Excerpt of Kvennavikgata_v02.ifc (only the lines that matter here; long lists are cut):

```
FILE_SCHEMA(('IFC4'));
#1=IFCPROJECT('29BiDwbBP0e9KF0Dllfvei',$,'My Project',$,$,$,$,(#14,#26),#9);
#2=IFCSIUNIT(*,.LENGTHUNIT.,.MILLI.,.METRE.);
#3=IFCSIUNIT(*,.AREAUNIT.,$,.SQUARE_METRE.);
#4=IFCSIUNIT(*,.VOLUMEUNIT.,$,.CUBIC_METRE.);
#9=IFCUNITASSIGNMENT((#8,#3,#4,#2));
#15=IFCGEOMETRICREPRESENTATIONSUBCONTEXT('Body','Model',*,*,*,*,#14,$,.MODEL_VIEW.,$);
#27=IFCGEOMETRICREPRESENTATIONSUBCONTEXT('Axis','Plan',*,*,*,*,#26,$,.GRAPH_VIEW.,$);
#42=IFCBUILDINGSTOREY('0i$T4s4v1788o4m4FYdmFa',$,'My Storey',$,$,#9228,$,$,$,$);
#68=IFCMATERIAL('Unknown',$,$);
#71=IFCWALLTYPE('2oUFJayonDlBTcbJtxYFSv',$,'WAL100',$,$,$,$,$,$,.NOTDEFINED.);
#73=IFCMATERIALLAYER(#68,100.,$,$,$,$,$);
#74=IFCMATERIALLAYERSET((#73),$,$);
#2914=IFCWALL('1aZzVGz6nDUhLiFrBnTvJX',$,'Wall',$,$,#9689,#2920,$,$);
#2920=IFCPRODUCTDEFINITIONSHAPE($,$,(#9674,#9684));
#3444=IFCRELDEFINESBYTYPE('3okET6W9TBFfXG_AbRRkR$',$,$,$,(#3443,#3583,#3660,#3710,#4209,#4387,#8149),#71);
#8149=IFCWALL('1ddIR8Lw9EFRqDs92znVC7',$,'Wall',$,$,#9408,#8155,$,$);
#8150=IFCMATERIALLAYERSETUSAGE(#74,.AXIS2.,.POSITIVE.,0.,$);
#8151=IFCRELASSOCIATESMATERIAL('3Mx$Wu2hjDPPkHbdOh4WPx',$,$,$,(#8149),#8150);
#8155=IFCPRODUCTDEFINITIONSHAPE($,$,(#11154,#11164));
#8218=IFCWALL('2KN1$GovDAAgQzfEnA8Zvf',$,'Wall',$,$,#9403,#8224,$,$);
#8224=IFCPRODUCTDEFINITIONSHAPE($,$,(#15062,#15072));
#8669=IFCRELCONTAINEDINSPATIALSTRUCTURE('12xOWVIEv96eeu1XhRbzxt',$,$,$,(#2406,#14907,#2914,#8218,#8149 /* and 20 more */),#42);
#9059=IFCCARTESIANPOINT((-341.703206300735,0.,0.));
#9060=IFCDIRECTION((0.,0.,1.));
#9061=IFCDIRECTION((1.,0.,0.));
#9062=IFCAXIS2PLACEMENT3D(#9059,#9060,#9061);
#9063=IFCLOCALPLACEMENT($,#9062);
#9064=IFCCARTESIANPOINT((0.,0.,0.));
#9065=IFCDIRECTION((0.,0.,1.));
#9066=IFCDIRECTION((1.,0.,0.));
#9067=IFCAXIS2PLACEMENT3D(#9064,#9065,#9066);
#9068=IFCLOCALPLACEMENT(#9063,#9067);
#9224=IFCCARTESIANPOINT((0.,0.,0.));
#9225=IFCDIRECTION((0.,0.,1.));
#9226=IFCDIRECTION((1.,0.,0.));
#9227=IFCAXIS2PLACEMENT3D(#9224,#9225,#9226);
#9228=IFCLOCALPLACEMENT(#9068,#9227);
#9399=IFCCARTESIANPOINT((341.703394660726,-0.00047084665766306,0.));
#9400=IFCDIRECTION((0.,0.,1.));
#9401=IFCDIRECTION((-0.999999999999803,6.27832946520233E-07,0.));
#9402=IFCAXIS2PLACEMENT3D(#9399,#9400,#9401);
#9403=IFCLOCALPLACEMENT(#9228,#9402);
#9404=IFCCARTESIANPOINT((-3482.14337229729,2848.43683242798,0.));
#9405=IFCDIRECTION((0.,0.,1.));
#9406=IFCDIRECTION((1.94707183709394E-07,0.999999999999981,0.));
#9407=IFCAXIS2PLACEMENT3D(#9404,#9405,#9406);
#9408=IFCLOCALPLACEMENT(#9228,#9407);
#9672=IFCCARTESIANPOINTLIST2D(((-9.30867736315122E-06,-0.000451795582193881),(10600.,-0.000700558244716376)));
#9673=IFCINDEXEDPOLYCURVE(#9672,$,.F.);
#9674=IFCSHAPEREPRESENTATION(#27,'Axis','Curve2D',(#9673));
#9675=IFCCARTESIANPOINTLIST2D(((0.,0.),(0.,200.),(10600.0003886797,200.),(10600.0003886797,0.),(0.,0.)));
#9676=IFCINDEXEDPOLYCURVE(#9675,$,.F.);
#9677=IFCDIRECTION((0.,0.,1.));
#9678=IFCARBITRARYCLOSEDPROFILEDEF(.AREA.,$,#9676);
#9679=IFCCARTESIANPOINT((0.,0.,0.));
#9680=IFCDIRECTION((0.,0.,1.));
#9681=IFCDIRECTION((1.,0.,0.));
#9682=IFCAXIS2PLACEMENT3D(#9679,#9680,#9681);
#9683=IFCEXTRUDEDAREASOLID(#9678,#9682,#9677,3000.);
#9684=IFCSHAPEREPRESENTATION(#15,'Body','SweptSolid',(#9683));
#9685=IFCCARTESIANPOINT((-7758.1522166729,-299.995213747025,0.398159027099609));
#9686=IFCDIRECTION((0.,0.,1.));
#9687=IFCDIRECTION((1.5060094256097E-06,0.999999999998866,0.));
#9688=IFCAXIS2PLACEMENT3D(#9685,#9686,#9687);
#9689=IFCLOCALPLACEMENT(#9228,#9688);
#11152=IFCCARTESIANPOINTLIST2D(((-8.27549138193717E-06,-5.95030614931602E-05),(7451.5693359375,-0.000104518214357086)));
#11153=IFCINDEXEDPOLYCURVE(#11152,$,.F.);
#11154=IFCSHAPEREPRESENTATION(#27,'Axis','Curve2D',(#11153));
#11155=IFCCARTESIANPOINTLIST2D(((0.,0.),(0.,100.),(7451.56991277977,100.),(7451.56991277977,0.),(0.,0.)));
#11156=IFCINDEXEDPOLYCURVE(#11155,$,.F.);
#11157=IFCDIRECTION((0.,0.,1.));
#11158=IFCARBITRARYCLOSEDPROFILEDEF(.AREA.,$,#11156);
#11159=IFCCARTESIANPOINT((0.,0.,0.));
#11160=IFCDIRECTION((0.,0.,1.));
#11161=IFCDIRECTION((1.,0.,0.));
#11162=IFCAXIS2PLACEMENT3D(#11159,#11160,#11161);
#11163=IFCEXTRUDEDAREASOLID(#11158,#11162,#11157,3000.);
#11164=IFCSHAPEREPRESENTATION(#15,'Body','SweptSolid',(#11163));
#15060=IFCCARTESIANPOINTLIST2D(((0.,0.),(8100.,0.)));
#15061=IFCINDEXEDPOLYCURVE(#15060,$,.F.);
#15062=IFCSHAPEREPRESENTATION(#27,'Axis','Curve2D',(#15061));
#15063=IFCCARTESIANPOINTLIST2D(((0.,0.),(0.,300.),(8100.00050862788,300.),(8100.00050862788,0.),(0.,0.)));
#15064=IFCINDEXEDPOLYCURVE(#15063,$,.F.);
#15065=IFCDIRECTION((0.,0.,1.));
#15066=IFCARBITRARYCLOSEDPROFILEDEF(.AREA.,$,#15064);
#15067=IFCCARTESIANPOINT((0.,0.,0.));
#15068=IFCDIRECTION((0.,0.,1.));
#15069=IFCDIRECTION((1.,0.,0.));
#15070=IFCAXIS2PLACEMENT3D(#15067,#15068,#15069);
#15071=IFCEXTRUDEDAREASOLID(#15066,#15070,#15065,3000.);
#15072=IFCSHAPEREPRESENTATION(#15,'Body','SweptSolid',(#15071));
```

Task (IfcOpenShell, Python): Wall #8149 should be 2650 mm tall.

```python
import ifcopenshell
import ifcopenshell.geom
import ifcopenshell.util.representation
import ifcopenshell.util.shape
import ifcopenshell.util.unit

model = ifcopenshell.open("Kvennavikgata_v02.ifc")
unit_scale = ifcopenshell.util.unit.calculate_unit_scale(model)
settings = ifcopenshell.geom.settings()


def volume(element):
    """Net volume in cubic metres, openings subtracted."""
    shape = ifcopenshell.geom.create_shape(settings, element)
    return ifcopenshell.util.shape.get_volume(shape.geometry)


wall = model.by_guid("1ddIR8Lw9EFRqDs92znVC7")
before = volume(wall)

body = ifcopenshell.util.representation.get_representation(wall, "Model", "Body")
solid = body.Items[0]
old_height = solid.Depth
solid.Depth = 2.65 / unit_scale
after = volume(wall)

print(f"height {old_height:g} -> {solid.Depth:g}, volume {before:.3f} -> {after:.3f} m3")

model.write("Kvennavikgata_v02_rev.ifc")
```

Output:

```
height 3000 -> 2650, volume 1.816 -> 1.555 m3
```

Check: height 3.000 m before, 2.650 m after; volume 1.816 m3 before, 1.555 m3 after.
